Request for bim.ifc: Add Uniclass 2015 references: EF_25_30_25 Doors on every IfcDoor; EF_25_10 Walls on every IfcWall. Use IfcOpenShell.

First a look at what the model holds.

```python
import ifcopenshell

model = ifcopenshell.open("bim.ifc")
print(model.schema)
print("classifications:", [c.Name for c in model.by_type("IfcClassification")])
for ifc_class in ("IfcDoor", "IfcRoof", "IfcStair", "IfcWall", "IfcWindow"):
    print(ifc_class, len(model.by_type(ifc_class)))
```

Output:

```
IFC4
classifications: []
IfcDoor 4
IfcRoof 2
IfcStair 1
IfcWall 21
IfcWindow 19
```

```python
import ifcopenshell
import ifcopenshell.api.classification

model = ifcopenshell.open("bim.ifc")

system = ifcopenshell.api.classification.add_classification(model, classification="Uniclass 2015")

codes = {
    "IfcDoor": ("EF_25_30_25", "Doors"),
    "IfcWall": ("EF_25_10", "Walls"),
}
for ifc_class, (code, name) in codes.items():
    products = model.by_type(ifc_class)
    ifcopenshell.api.classification.add_reference(
        model, products=products, classification=system, identification=code, name=name
    )
    print(code, len(products))

model.write("bim-out.ifc")
```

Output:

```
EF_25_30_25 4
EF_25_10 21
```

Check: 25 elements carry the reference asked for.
